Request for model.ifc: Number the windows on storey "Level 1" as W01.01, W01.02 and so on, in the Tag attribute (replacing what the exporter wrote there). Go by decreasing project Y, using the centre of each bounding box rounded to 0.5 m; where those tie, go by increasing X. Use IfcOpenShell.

First a look at what the model holds.

```python
import ifcopenshell
import ifcopenshell.util.element
import ifcopenshell.util.placement

model = ifcopenshell.open("model.ifc")
print(model.schema)
storey = next(s for s in model.by_type("IfcBuildingStorey") if s.Name == "Level 1")
windows = [e for e in ifcopenshell.util.element.get_decomposition(storey) if e.is_a("IfcWindow")]
for e in sorted(windows, key=lambda e: e.id()):
    origin = ifcopenshell.util.placement.get_local_placement(e.ObjectPlacement)[:3, 3]
    print(e.id(), e.Tag, e.Name, origin.round(2) + 0.0, sep=" | ")
```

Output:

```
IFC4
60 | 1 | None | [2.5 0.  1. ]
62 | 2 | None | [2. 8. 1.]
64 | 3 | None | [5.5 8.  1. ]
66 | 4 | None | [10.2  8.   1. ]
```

```python
import ifcopenshell
import ifcopenshell.geom
import ifcopenshell.util.element
import ifcopenshell.util.shape

model = ifcopenshell.open("model.ifc")
settings = ifcopenshell.geom.settings()
settings.set("use-world-coords", True)


def centre(element):
    shape = ifcopenshell.geom.create_shape(settings, element)
    return ifcopenshell.util.shape.get_bbox_centroid(shape.geometry)


storey = next(s for s in model.by_type("IfcBuildingStorey") if s.Name == "Level 1")
windows = [e for e in ifcopenshell.util.element.get_decomposition(storey) if e.is_a("IfcWindow")]

# Insertion points can sit at a corner or the storey origin, so sort by the geometry (in metres).
centres = {e: centre(e) for e in windows}
windows.sort(key=lambda e: (-round(centres[e][1] / 0.5), centres[e][0]))

for i, e in enumerate(windows, start=1):
    number = f"W01.{i:02d}"
    e.Tag = number
    print(e.id(), number)

model.write("model-out.ifc")
```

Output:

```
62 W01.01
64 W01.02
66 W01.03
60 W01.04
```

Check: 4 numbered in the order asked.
